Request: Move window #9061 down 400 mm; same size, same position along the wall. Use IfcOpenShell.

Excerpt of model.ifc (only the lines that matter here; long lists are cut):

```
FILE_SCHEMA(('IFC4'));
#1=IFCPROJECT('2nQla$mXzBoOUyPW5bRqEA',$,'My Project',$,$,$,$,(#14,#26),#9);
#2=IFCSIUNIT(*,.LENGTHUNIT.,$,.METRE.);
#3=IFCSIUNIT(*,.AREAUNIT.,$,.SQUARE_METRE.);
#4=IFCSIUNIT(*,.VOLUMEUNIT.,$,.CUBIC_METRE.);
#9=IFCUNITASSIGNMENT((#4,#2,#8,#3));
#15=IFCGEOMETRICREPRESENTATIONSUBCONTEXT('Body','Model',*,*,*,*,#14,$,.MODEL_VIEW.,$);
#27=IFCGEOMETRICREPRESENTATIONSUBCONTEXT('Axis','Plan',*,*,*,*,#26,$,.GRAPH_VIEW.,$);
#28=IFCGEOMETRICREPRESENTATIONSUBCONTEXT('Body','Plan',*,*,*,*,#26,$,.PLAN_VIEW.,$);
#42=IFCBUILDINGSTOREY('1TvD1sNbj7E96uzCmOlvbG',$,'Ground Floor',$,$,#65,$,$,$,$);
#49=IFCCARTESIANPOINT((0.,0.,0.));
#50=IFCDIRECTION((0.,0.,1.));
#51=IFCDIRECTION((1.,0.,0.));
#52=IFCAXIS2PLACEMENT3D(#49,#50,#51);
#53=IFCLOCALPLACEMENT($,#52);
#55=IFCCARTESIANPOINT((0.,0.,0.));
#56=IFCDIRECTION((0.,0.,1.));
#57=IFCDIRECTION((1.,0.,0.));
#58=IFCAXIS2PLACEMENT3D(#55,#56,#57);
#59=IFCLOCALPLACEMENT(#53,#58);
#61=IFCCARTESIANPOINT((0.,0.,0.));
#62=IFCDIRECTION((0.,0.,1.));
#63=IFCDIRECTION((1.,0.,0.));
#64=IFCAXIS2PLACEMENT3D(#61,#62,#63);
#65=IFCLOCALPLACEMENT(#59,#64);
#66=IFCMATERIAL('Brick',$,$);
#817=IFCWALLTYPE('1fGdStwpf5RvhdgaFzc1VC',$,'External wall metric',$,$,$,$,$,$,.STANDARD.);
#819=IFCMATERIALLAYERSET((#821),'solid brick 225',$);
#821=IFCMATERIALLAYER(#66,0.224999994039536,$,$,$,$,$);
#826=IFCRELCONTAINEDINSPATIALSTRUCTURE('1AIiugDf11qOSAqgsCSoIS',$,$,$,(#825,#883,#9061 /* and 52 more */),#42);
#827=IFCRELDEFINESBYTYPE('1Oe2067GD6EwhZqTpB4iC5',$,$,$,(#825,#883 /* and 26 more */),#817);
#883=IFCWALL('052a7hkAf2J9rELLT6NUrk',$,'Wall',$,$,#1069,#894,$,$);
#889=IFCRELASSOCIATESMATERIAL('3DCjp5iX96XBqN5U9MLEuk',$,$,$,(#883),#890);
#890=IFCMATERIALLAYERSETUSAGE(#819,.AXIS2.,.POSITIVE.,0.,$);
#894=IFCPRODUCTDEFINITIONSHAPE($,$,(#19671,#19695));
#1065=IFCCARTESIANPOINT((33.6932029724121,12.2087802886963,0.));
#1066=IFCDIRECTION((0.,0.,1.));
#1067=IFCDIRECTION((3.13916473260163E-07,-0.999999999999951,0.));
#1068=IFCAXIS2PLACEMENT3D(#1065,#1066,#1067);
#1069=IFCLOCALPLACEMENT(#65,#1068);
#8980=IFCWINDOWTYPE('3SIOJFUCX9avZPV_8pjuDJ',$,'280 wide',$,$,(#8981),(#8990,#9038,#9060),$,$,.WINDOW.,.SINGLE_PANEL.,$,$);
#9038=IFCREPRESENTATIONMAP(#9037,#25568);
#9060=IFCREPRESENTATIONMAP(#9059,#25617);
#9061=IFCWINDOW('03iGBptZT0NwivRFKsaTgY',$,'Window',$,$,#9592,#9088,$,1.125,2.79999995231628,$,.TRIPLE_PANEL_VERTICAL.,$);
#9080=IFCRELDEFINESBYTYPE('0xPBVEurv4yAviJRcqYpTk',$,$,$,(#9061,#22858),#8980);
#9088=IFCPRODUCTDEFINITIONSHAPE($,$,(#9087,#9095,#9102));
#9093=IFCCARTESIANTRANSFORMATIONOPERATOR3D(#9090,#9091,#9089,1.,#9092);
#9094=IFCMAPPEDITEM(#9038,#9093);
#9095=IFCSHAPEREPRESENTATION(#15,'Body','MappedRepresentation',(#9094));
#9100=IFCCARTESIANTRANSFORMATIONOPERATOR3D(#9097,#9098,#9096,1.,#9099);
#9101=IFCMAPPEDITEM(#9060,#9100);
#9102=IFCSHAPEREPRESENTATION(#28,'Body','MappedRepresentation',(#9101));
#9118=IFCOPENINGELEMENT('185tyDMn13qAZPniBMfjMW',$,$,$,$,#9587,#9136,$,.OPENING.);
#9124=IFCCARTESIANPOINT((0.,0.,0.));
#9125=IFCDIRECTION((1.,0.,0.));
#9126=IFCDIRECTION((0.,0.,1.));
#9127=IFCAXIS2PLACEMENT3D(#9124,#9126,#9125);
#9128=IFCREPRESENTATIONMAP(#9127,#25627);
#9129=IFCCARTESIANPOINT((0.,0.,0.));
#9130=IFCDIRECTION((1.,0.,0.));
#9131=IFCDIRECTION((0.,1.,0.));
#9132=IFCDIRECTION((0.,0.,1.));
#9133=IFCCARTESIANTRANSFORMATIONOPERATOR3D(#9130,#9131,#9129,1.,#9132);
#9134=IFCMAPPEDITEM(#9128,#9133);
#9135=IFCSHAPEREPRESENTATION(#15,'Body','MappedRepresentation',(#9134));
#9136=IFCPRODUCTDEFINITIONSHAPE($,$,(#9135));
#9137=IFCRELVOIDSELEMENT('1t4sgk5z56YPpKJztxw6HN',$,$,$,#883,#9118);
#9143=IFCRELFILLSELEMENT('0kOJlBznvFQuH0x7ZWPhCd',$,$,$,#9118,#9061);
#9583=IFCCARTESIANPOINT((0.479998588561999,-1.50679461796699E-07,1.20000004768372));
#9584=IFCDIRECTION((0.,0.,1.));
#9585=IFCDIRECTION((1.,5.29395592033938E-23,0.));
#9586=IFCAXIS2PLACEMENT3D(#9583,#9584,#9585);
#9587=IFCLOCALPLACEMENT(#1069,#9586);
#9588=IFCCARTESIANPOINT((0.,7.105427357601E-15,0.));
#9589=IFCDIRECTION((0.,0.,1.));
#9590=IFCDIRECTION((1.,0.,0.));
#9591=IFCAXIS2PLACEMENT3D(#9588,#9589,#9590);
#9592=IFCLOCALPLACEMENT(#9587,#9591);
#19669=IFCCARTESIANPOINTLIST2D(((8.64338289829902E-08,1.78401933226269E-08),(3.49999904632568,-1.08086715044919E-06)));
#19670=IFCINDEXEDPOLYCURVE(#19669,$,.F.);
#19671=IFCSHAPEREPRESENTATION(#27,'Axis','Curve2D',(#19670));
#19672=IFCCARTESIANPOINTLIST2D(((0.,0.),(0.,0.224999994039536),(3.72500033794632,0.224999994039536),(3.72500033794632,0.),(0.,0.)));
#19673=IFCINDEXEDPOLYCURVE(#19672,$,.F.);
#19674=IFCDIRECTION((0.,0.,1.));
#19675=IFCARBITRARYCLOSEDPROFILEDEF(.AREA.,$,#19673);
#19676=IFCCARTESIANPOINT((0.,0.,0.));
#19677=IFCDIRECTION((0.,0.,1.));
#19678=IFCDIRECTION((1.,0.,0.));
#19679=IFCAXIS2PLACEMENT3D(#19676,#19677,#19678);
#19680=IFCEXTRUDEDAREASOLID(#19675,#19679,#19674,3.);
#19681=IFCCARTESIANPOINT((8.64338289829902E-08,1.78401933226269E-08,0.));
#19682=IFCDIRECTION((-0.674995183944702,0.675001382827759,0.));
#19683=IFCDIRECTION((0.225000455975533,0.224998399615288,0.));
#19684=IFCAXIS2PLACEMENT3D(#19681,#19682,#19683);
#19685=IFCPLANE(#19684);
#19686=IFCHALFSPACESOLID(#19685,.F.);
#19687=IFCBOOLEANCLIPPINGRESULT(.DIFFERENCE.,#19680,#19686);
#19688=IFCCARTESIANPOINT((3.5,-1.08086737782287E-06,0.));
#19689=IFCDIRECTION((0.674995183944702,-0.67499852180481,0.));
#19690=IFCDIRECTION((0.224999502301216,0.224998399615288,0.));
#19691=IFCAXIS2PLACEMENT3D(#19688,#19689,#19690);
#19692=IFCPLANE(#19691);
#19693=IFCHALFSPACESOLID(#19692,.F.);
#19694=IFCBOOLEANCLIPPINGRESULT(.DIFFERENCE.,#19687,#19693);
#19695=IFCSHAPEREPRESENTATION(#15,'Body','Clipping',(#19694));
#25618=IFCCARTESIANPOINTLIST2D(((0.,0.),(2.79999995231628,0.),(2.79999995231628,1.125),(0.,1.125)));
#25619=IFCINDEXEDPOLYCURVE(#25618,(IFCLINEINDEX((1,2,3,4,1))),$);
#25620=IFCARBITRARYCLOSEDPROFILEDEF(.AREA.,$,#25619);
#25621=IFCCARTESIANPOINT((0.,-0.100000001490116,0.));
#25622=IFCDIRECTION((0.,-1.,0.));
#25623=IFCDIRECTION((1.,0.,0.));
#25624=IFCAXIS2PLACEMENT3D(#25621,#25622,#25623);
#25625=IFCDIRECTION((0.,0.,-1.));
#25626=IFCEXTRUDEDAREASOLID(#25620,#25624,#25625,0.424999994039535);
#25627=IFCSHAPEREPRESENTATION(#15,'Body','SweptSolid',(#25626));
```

```python
import numpy as np
import ifcopenshell
import ifcopenshell.api.geometry
import ifcopenshell.util.placement
import ifcopenshell.util.unit

model = ifcopenshell.open("model.ifc")
unit_scale = ifcopenshell.util.unit.calculate_unit_scale(model)

window = model.by_guid("03iGBptZT0NwivRFKsaTgY")
opening = window.FillsVoids[0].RelatingOpeningElement
dz = -0.4 / unit_scale

shift = np.array([0.0, 0.0, dz])
# The window is placed relative to its opening, so it follows when the opening moves.
matrix = ifcopenshell.util.placement.get_local_placement(opening.ObjectPlacement)
matrix[:3, 3] += shift
ifcopenshell.api.geometry.edit_object_placement(
    model, product=opening, matrix=matrix, is_si=False, should_transform_children=True
)

print(f"moved by {dz * unit_scale:+.3f} m")

model.write("model_updated.ifc")
```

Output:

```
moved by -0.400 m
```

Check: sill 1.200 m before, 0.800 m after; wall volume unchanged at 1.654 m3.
